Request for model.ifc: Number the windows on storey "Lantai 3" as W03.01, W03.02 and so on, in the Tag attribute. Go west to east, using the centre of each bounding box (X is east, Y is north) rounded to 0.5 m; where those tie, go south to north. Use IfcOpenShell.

First a look at what the model holds.

```python
import ifcopenshell
import ifcopenshell.util.element
import ifcopenshell.util.placement

model = ifcopenshell.open("model.ifc")
print(model.schema)
storey = next(s for s in model.by_type("IfcBuildingStorey") if s.Name == "Lantai 3")
windows = [e for e in ifcopenshell.util.element.get_decomposition(storey) if e.is_a("IfcWindow")]
for e in sorted(windows, key=lambda e: e.id()):
    origin = ifcopenshell.util.placement.get_local_placement(e.ObjectPlacement)[:3, 3]
    print(e.id(), e.Tag, e.Name, origin.round(2) + 0.0, sep=" | ")
```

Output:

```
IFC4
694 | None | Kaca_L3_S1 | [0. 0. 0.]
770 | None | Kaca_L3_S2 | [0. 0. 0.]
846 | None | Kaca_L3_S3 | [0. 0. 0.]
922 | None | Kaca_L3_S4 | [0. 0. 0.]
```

```python
import ifcopenshell
import ifcopenshell.geom
import ifcopenshell.util.element
import ifcopenshell.util.shape

model = ifcopenshell.open("model.ifc")
settings = ifcopenshell.geom.settings()
settings.set("use-world-coords", True)


def centre(element):
    shape = ifcopenshell.geom.create_shape(settings, element)
    return ifcopenshell.util.shape.get_bbox_centroid(shape.geometry)


storey = next(s for s in model.by_type("IfcBuildingStorey") if s.Name == "Lantai 3")
windows = [e for e in ifcopenshell.util.element.get_decomposition(storey) if e.is_a("IfcWindow")]

# Insertion points can sit at a corner or the storey origin, so sort by the geometry (in metres).
centres = {e: centre(e) for e in windows}
windows.sort(key=lambda e: (round(centres[e][0] / 0.5), centres[e][1]))

for i, e in enumerate(windows, start=1):
    number = f"W03.{i:02d}"
    e.Tag = number
    print(e.id(), number)

model.write("model-out.ifc")
```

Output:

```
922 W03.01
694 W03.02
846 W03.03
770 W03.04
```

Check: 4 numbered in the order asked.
